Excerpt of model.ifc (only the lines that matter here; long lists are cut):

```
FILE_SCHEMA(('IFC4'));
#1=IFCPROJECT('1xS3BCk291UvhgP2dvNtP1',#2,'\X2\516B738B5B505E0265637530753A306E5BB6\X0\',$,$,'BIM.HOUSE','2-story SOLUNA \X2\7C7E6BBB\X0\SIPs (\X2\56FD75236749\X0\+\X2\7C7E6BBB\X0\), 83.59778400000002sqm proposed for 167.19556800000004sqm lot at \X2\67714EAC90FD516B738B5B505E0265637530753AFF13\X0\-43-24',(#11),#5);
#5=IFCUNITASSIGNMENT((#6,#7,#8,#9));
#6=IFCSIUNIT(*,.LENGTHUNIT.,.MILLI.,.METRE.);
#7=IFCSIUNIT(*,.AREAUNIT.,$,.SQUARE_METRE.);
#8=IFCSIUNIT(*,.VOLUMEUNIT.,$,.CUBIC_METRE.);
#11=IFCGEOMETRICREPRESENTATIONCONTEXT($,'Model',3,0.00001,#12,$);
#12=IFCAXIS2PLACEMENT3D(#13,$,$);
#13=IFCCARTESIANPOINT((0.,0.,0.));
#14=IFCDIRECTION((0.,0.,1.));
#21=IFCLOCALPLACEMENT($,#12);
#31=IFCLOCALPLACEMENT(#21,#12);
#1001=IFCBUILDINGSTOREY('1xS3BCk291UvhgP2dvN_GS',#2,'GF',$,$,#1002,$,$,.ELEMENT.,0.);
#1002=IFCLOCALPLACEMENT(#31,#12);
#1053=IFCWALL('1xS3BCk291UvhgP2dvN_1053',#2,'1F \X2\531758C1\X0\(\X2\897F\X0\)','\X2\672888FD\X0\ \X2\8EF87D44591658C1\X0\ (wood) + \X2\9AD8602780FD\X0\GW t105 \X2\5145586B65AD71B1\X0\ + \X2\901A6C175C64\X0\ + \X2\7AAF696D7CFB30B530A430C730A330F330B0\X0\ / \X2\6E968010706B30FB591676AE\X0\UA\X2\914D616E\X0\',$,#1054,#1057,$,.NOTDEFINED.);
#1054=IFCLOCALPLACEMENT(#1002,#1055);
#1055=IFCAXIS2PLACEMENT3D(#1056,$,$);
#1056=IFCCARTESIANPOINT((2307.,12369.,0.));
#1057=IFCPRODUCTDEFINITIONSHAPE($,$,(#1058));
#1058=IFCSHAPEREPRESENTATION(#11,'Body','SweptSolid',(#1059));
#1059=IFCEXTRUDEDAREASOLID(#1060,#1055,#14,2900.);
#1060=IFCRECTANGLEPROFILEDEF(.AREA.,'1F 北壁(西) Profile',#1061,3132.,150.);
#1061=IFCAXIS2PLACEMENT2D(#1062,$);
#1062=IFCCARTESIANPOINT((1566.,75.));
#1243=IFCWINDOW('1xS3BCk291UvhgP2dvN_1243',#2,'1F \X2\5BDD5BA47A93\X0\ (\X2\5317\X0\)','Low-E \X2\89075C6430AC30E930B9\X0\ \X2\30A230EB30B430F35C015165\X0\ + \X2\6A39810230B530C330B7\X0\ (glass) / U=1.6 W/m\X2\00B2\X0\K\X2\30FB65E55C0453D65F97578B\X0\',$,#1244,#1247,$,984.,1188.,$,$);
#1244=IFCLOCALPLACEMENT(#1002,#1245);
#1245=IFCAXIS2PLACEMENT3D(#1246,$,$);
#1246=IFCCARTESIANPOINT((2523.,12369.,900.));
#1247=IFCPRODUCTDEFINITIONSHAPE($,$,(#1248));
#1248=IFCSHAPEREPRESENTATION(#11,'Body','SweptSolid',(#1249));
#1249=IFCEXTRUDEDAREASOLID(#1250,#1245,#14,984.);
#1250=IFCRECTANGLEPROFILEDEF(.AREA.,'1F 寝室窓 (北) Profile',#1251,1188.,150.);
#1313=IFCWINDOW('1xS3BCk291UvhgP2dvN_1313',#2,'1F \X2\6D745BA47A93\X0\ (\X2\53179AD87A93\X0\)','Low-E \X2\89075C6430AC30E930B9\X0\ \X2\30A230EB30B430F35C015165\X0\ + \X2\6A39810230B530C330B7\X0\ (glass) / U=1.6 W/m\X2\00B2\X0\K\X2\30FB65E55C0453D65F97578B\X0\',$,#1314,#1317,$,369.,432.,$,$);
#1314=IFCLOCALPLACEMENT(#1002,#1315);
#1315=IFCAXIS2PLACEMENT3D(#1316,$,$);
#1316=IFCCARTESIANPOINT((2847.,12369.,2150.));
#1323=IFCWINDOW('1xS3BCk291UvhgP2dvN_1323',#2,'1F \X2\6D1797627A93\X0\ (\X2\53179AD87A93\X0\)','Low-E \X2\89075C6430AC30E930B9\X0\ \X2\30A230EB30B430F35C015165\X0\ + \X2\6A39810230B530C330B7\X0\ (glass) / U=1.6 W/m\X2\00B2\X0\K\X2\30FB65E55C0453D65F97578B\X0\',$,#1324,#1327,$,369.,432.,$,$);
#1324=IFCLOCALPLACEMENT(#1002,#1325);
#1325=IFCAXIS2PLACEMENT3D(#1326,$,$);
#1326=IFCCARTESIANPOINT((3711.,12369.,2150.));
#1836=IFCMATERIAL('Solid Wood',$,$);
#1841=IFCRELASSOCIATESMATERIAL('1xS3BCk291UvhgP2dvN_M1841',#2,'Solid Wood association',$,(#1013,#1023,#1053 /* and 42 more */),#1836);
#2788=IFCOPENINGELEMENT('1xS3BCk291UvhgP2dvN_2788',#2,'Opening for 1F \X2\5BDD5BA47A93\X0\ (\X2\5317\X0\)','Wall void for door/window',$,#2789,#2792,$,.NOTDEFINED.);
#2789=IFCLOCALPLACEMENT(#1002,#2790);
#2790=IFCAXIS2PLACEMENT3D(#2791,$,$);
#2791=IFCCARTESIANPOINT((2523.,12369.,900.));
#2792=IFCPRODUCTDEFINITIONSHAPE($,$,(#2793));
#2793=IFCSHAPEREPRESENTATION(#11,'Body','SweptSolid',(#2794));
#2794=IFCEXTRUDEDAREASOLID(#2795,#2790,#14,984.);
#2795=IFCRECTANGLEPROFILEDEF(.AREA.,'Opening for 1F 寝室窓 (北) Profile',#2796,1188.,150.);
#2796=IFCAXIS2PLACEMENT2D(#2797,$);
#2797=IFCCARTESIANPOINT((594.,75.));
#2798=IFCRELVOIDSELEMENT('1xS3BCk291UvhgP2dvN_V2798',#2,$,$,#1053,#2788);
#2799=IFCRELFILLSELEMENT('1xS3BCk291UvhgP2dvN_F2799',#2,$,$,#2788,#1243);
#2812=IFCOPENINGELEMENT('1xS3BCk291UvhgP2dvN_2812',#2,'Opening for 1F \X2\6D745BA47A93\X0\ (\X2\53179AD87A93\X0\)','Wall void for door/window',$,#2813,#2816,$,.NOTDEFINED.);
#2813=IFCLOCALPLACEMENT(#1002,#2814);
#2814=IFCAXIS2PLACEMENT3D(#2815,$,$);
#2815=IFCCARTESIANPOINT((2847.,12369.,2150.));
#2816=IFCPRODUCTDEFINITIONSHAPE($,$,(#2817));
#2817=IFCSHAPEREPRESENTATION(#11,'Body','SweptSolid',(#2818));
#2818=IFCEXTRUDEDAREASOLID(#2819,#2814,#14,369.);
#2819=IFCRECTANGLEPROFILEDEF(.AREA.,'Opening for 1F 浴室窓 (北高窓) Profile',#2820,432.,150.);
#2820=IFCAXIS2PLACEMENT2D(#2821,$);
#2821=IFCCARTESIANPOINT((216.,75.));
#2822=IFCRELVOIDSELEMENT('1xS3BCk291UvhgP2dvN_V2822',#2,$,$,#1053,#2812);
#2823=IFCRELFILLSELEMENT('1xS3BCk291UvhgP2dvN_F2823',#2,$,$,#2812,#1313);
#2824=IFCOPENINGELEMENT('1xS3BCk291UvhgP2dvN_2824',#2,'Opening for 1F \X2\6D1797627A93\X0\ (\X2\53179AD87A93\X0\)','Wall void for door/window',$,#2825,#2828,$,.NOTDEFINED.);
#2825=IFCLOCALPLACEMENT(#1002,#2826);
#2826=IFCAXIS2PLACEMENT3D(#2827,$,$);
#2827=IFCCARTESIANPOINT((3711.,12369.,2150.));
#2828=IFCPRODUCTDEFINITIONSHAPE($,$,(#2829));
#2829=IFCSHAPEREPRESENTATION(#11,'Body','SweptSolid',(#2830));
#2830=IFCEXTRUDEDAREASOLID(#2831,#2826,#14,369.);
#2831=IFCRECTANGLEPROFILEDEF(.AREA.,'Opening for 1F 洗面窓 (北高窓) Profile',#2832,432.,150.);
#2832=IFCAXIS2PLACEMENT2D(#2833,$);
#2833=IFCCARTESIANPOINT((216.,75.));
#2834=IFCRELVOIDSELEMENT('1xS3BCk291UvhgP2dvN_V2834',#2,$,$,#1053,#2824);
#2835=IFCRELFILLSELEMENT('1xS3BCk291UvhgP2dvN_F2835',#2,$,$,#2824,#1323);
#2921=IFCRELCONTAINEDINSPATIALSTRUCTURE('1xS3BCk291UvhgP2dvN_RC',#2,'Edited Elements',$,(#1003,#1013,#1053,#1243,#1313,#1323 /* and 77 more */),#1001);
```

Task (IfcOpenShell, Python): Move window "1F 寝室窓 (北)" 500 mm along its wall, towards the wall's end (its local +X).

```python
import ifcopenshell
import ifcopenshell.api.geometry
import ifcopenshell.util.placement
import ifcopenshell.util.unit

model = ifcopenshell.open("model.ifc")
unit_scale = ifcopenshell.util.unit.calculate_unit_scale(model)

window = model.by_guid("1xS3BCk291UvhgP2dvN_1243")
opening = window.FillsVoids[0].RelatingOpeningElement
wall = opening.VoidsElements[0].RelatingBuildingElement

wall_matrix = ifcopenshell.util.placement.get_local_placement(wall.ObjectPlacement)
shift = wall_matrix[:3, 0] * 0.5 / unit_scale
before = ifcopenshell.util.placement.get_local_placement(window.ObjectPlacement)[:3, 3].copy()

# The window is not placed relative to its opening, so move both.
for product in (opening, window):
    matrix = ifcopenshell.util.placement.get_local_placement(product.ObjectPlacement)
    matrix[:3, 3] += shift
    ifcopenshell.api.geometry.edit_object_placement(model, product=product, matrix=matrix, is_si=False)

after = ifcopenshell.util.placement.get_local_placement(window.ObjectPlacement)[:3, 3]
print("window moved by", (after - before).round(3) + 0.0)

model.write("model-out.ifc")
```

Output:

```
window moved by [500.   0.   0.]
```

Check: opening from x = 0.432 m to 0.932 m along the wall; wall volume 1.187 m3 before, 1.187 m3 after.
